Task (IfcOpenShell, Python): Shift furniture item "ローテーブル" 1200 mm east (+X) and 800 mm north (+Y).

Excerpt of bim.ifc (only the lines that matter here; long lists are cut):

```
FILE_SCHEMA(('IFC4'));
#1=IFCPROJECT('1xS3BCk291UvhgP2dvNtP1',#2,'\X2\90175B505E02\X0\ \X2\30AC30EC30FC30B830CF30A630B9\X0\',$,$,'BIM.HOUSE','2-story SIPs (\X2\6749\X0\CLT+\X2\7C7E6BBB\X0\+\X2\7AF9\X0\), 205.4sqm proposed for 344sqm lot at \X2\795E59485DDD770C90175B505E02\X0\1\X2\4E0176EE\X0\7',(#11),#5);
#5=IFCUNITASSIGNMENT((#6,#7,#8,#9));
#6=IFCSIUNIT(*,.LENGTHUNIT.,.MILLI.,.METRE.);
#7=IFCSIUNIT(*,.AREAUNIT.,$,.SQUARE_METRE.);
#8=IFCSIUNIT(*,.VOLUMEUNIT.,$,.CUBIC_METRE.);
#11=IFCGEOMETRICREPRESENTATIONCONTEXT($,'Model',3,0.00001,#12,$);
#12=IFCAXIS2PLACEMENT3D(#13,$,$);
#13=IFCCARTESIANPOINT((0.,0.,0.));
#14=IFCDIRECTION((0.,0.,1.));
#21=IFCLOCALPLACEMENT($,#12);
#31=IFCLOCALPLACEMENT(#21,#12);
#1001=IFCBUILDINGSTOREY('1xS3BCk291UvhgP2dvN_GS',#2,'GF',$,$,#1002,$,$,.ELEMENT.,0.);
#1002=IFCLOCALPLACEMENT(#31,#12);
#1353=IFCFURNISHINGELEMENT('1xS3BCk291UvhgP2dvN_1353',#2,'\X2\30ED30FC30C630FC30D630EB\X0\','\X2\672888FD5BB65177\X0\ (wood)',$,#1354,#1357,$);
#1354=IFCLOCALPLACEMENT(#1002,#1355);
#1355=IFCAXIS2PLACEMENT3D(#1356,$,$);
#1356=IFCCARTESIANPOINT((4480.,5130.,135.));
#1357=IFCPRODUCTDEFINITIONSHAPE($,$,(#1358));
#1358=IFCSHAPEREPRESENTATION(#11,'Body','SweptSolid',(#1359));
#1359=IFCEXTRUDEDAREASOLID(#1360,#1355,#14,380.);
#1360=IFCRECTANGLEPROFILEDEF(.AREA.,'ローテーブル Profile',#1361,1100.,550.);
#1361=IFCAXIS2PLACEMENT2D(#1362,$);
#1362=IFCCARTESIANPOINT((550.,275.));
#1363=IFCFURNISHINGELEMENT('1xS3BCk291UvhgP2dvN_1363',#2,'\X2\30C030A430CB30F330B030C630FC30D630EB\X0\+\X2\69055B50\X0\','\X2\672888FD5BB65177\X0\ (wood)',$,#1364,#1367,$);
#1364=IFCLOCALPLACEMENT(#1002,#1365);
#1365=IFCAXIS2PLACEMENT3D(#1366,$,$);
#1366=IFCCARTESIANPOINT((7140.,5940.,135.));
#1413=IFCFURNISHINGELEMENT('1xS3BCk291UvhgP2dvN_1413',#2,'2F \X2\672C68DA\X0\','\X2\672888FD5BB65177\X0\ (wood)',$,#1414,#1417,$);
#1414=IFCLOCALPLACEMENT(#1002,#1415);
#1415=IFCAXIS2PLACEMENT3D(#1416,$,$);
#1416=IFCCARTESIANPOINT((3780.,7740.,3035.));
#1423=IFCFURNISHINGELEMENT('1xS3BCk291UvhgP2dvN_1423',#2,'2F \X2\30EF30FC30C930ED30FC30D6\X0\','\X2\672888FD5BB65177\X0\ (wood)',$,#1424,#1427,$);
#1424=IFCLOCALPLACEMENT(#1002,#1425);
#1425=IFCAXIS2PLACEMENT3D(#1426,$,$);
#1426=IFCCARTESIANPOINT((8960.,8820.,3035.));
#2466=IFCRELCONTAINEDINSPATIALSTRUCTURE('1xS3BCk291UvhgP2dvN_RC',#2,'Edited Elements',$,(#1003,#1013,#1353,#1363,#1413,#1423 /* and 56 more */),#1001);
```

```python
import ifcopenshell
import ifcopenshell.api.geometry
import ifcopenshell.util.placement
import ifcopenshell.util.unit

model = ifcopenshell.open("bim.ifc")
unit_scale = ifcopenshell.util.unit.calculate_unit_scale(model)

item = model.by_guid("1xS3BCk291UvhgP2dvN_1353")
matrix = ifcopenshell.util.placement.get_local_placement(item.ObjectPlacement)
matrix[0, 3] += 1.2 / unit_scale
matrix[1, 3] += 0.8 / unit_scale
ifcopenshell.api.geometry.edit_object_placement(model, product=item, matrix=matrix, is_si=False)

print(ifcopenshell.util.placement.get_local_placement(item.ObjectPlacement).round(3) + 0.0)

model.write("bim-out.ifc")
```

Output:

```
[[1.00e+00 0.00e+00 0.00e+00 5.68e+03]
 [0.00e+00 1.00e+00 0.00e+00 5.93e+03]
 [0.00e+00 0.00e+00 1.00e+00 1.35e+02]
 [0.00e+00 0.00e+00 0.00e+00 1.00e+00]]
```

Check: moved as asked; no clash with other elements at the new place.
